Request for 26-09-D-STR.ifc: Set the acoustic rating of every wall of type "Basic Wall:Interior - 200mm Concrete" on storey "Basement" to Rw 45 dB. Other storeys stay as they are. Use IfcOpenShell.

First a look at what the model holds.

```python
import ifcopenshell
import ifcopenshell.util.element

model = ifcopenshell.open("26-09-D-STR.ifc")
print(model.schema)
storey = next(s for s in model.by_type("IfcBuildingStorey") if s.Name == "Basement")
walls = [e for e in ifcopenshell.util.element.get_decomposition(storey) if e.is_a("IfcWall")]
seen = {}
for e in walls:
    element_type = ifcopenshell.util.element.get_type(e)
    key = (element_type.Name if element_type != e and element_type else None, ifcopenshell.util.element.get_pset(e, "Pset_WallCommon", "AcousticRating"))
    seen[key] = seen.get(key, 0) + 1
for (name, value), count in sorted(seen.items(), key=str):
    print(count, "x", name, "|", value)
```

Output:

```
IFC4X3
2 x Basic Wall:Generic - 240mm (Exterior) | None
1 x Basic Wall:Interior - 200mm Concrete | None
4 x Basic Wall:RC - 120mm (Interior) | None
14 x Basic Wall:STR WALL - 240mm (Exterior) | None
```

```python
import ifcopenshell
import ifcopenshell.api.pset
import ifcopenshell.util.element

model = ifcopenshell.open("26-09-D-STR.ifc")

storey = next(s for s in model.by_type("IfcBuildingStorey") if s.Name == "Basement")
walls = [e for e in ifcopenshell.util.element.get_decomposition(storey) if e.is_a("IfcWall")]

count = 0
for e in walls:
    element_type = ifcopenshell.util.element.get_type(e)
    if element_type in (None, e) or element_type.Name != "Basic Wall:Interior - 200mm Concrete":
        continue
    # add_pset returns the element's existing set when there is one.
    pset = ifcopenshell.api.pset.add_pset(model, product=e, name="Pset_WallCommon")
    ifcopenshell.api.pset.edit_pset(model, pset=pset, properties={"AcousticRating": "Rw 45 dB"})
    count += 1

print(count, "walls updated")

model.write("26-09-D-STR_edited.ifc")
```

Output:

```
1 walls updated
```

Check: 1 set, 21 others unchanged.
